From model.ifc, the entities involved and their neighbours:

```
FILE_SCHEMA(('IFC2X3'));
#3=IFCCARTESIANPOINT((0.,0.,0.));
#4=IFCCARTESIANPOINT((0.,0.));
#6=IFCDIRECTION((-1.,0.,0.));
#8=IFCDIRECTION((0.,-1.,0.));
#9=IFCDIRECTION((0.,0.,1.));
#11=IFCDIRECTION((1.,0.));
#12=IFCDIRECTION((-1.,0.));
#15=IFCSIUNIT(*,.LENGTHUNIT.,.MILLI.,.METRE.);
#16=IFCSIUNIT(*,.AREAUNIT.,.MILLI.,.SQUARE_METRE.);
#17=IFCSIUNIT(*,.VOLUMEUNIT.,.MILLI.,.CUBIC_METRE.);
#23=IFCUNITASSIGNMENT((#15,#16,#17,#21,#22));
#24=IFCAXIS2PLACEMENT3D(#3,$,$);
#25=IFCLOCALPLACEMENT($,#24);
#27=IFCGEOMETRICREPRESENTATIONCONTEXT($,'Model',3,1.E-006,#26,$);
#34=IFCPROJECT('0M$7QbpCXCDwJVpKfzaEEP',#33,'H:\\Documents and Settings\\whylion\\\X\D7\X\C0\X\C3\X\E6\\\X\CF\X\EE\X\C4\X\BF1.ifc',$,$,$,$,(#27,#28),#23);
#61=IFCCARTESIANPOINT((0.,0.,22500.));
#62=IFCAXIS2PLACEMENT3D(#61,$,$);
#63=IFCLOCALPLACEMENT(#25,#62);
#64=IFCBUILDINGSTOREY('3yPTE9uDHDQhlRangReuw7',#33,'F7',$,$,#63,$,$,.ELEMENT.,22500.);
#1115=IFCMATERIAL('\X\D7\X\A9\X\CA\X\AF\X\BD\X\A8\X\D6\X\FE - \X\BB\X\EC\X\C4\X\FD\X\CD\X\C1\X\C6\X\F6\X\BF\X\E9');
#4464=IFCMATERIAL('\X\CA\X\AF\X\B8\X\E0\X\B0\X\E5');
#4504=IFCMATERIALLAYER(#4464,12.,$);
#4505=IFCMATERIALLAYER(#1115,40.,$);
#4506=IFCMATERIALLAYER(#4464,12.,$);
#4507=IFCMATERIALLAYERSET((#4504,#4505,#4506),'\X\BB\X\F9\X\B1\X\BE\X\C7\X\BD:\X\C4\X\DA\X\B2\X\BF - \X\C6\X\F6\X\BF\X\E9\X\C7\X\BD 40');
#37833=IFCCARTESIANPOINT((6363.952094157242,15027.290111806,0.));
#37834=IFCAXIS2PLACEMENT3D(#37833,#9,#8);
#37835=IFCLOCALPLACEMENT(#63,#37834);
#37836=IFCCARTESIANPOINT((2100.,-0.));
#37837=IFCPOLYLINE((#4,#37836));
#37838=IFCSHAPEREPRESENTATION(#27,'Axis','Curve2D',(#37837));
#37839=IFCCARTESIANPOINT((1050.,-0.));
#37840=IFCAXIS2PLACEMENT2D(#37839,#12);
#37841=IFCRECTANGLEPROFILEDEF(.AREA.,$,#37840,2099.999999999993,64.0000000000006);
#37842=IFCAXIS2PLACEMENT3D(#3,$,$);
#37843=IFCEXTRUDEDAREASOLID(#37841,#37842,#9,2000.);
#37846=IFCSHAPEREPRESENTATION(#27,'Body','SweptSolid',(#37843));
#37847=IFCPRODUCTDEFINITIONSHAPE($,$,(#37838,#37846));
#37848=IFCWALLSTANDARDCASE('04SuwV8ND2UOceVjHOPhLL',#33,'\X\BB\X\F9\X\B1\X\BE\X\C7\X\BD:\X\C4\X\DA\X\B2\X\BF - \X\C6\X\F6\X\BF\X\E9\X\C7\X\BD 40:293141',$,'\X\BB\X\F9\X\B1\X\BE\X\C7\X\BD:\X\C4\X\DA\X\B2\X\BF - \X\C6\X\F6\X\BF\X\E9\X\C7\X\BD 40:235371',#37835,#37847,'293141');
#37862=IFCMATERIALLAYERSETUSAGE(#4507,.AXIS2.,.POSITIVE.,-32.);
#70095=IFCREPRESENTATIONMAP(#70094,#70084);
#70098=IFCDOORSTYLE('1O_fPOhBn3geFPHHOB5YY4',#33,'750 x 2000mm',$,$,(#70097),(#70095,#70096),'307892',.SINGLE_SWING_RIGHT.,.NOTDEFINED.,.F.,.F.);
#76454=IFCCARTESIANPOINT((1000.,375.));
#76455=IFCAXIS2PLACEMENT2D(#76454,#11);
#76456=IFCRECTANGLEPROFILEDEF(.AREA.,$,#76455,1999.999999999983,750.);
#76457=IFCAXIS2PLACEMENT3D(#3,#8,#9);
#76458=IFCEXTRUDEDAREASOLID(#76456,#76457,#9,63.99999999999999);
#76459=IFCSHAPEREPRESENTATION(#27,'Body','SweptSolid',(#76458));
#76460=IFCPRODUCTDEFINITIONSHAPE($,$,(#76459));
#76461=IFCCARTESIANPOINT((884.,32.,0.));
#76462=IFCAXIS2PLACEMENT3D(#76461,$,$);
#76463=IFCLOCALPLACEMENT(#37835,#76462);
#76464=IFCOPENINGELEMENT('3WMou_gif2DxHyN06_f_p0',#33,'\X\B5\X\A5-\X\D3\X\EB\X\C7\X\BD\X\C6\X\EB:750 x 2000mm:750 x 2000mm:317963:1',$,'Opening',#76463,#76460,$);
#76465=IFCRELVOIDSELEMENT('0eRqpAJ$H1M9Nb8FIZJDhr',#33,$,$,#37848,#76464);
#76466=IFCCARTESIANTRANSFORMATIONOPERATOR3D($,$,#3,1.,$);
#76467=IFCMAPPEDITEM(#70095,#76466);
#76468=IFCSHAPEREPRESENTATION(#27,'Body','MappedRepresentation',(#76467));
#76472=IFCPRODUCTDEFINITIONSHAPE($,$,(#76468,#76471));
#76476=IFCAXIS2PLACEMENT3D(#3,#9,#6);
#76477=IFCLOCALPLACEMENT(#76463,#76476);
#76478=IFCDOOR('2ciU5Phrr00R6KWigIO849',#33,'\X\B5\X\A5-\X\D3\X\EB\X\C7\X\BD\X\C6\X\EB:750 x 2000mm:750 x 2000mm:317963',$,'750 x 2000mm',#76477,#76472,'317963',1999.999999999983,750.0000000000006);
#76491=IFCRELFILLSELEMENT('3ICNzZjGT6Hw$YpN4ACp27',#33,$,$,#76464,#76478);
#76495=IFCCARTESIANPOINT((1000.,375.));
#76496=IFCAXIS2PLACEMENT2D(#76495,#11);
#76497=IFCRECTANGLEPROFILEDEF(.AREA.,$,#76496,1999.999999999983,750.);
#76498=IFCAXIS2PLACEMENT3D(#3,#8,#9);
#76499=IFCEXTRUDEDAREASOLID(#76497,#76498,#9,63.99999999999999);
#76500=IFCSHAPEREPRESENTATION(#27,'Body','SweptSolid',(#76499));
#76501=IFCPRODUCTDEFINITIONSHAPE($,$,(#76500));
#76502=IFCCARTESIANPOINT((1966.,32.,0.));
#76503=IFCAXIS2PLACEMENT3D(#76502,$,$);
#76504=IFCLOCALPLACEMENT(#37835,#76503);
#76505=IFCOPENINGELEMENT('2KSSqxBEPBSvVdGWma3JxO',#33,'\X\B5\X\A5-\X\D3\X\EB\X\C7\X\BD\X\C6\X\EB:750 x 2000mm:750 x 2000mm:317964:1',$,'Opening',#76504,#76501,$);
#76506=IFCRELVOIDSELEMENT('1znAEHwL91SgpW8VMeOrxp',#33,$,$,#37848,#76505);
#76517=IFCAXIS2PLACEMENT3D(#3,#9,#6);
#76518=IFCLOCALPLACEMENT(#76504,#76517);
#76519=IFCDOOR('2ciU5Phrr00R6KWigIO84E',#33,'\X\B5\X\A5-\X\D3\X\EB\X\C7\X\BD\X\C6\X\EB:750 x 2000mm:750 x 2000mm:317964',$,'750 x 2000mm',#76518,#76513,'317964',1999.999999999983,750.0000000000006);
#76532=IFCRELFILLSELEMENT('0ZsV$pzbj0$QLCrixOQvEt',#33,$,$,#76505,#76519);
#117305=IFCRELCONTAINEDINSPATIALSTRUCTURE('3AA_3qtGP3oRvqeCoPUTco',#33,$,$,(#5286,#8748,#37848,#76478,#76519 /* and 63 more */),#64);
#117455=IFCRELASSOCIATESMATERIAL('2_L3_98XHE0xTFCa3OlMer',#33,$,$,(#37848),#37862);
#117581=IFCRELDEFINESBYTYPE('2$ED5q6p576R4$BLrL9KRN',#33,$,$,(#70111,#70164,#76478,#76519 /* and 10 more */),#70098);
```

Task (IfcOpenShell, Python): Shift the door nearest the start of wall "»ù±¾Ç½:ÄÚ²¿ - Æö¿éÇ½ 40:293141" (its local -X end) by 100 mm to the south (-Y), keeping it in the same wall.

```python
import ifcopenshell
import ifcopenshell.api.geometry
import ifcopenshell.util.placement

model = ifcopenshell.open("model.ifc")

door = model.by_guid("2ciU5Phrr00R6KWigIO849")
opening = door.FillsVoids[0].RelatingOpeningElement
wall = opening.VoidsElements[0].RelatingBuildingElement

wall_matrix = ifcopenshell.util.placement.get_local_placement(wall.ObjectPlacement)
shift = wall_matrix[:3, 0] * 100.0
before = ifcopenshell.util.placement.get_local_placement(door.ObjectPlacement)[:3, 3].copy()

# The door is placed relative to its opening, so it follows when the opening moves.
matrix = ifcopenshell.util.placement.get_local_placement(opening.ObjectPlacement)
matrix[:3, 3] += shift
ifcopenshell.api.geometry.edit_object_placement(
    model, product=opening, matrix=matrix, is_si=False, should_transform_children=True
)

after = ifcopenshell.util.placement.get_local_placement(door.ObjectPlacement)[:3, 3]
print("door moved by", (after - before).round(3) + 0.0)

model.write("model_updated.ifc")
```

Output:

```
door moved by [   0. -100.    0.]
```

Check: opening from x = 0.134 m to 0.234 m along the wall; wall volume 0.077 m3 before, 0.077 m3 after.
